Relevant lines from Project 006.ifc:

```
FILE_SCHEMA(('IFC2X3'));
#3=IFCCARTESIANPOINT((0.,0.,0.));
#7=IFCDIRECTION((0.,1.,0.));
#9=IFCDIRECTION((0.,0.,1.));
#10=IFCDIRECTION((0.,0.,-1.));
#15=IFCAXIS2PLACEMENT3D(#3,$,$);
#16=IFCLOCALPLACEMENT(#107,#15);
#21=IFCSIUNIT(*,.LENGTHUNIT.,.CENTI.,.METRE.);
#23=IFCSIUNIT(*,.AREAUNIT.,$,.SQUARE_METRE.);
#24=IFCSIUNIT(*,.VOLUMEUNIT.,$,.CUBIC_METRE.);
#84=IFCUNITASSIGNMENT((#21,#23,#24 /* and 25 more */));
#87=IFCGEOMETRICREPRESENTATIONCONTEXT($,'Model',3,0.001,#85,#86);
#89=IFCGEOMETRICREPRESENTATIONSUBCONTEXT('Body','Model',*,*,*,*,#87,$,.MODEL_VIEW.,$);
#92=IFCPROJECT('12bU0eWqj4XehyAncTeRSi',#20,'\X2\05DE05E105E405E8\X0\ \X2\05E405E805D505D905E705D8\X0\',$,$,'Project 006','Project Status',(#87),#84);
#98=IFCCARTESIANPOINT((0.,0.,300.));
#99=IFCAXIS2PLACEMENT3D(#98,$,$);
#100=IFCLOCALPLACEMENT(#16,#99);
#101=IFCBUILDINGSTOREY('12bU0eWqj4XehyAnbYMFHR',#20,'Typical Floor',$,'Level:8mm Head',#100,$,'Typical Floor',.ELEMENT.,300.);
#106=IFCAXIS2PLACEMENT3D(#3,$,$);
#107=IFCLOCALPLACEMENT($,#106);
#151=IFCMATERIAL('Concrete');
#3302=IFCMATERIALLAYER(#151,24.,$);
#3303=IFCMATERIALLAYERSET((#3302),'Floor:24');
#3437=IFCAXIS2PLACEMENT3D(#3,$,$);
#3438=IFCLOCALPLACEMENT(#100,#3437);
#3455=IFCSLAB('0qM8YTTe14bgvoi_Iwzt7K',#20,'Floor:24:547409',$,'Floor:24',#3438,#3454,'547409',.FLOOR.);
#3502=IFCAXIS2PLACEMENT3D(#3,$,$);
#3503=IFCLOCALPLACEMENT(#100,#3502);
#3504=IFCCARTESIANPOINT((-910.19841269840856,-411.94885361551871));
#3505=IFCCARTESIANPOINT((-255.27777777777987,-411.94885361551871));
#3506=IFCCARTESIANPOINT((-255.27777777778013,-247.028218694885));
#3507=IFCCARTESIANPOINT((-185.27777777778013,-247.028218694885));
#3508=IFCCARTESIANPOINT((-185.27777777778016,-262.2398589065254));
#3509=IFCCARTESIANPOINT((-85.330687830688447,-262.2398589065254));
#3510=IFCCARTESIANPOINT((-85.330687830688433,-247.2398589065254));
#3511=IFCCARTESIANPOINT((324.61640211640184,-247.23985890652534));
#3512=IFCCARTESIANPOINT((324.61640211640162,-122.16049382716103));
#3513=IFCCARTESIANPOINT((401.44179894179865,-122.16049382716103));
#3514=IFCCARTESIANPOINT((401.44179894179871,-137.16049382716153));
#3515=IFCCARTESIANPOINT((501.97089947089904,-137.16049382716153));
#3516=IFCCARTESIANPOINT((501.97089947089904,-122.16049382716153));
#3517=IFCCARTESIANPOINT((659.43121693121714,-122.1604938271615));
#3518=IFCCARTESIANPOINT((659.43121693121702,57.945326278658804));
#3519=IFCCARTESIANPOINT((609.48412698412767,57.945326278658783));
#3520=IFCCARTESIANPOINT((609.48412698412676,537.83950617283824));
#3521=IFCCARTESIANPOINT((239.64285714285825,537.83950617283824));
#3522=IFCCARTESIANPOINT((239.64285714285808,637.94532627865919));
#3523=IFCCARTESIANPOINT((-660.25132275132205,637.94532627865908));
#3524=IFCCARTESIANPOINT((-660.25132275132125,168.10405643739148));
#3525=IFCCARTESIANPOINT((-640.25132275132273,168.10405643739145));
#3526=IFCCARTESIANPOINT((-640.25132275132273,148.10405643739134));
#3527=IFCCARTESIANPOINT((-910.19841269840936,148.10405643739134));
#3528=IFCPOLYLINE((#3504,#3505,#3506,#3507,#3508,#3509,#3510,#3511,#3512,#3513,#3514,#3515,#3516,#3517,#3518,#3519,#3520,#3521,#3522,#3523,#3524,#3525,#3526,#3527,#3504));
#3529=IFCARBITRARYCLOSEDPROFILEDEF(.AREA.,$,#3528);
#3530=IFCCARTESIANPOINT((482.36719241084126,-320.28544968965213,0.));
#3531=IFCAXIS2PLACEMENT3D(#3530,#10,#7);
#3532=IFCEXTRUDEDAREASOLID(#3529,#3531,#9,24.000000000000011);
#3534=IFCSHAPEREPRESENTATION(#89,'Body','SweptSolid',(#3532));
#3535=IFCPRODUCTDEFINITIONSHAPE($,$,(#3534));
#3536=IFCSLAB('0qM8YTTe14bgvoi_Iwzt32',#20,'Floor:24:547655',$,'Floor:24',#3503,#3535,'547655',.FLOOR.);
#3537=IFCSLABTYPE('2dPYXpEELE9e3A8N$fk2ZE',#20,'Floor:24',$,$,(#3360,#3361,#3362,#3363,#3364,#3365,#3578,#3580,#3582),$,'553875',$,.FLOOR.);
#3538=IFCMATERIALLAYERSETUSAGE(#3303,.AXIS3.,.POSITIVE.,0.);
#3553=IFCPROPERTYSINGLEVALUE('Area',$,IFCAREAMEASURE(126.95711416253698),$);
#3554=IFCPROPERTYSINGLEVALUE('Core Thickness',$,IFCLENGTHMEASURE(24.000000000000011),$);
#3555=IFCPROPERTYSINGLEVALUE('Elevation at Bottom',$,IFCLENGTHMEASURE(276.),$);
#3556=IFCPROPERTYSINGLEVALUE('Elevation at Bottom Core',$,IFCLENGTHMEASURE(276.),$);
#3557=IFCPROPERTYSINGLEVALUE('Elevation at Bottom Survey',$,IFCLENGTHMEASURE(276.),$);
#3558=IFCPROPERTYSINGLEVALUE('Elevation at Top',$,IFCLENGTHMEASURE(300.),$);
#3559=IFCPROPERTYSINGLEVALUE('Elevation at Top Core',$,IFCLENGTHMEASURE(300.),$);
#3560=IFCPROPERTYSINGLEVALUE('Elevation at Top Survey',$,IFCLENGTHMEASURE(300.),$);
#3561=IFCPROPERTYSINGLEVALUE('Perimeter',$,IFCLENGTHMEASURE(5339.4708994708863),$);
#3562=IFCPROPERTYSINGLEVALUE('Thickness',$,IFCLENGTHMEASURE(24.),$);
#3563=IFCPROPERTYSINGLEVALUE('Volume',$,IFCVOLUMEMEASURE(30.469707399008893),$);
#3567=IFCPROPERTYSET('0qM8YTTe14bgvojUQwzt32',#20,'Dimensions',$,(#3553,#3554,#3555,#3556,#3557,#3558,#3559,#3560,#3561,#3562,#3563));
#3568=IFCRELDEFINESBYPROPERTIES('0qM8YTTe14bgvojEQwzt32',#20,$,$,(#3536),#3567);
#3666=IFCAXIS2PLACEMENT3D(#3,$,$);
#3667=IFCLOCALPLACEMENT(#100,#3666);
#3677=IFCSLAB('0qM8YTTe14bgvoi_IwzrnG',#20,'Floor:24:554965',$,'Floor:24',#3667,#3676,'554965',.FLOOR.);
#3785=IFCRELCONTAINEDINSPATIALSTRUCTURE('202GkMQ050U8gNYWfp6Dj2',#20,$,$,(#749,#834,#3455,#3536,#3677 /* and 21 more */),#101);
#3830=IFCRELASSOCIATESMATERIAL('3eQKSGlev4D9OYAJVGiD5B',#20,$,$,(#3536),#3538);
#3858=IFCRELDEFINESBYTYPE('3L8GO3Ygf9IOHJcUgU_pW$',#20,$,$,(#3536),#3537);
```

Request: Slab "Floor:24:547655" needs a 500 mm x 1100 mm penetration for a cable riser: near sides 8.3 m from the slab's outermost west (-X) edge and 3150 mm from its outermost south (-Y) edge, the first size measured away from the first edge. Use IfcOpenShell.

```python
import numpy as np
import ifcopenshell
import ifcopenshell.api.feature
import ifcopenshell.api.geometry
import ifcopenshell.api.pset
import ifcopenshell.api.root
import ifcopenshell.geom
import ifcopenshell.util.element
import ifcopenshell.util.placement
import ifcopenshell.util.representation
import ifcopenshell.util.shape
import ifcopenshell.util.unit

model = ifcopenshell.open("Project 006.ifc")
unit_scale = ifcopenshell.util.unit.calculate_unit_scale(model)
area_scale = ifcopenshell.util.unit.calculate_unit_scale(model, "AREAUNIT")
volume_scale = ifcopenshell.util.unit.calculate_unit_scale(model, "VOLUMEUNIT")
settings = ifcopenshell.geom.settings()


def volume(element):
    """Net volume in cubic metres, openings subtracted."""
    shape = ifcopenshell.geom.create_shape(settings, element)
    return ifcopenshell.util.shape.get_volume(shape.geometry)


slab = model.by_guid("0qM8YTTe14bgvoi_Iwzt32")
before = volume(slab)

# Extent in the slab's own axes, in metres. The edges named are its -X and -Y sides.
slab_shape = ifcopenshell.geom.create_shape(settings, slab)
vertices = ifcopenshell.util.shape.get_vertices(slab_shape.geometry)
x_min, y_min, bottom = vertices.min(axis=0)
top = vertices[:, 2].max()

opening = ifcopenshell.api.root.create_entity(model, ifc_class="IfcOpeningElement", name="Cable riser opening")
context = ifcopenshell.util.representation.get_context(model, "Model", "Body", "MODEL_VIEW")
width, depth = 0.5, 1.1
outline = [(0.0, 0.0), (width, 0.0), (width, depth), (0.0, depth), (0.0, 0.0)]
# Overshoot both faces by 50 mm so the cut is clean.
shape = ifcopenshell.api.geometry.add_slab_representation(
    model, context=context, depth=top - bottom + 0.1, polyline=outline
)
ifcopenshell.api.geometry.assign_representation(model, product=opening, representation=shape)

matrix = ifcopenshell.util.placement.get_local_placement(slab.ObjectPlacement)
matrix[:, 3] = matrix @ np.append(np.array([x_min + 8.3, y_min + 3.15, bottom - 0.05]) / unit_scale, 1.0)
ifcopenshell.api.geometry.edit_object_placement(model, product=opening, matrix=matrix, is_si=False)
ifcopenshell.api.feature.add_feature(model, feature=opening, element=slab)

after = volume(slab)

# Update the slab's stored quantities.
pset = model.by_id(ifcopenshell.util.element.get_pset(slab, "Dimensions", should_inherit=False)["id"])
ifcopenshell.api.pset.edit_pset(model, pset=pset, properties={
    "Area": model.create_entity("IfcAreaMeasure", after / (top - bottom) / area_scale),
    "Volume": model.create_entity("IfcVolumeMeasure", after / volume_scale),
})

print(f"slab volume {before:.3f} -> {after:.3f} m3")

model.write("Project 006_updated.ifc")
```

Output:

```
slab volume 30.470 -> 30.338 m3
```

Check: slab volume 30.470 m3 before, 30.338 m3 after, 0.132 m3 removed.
